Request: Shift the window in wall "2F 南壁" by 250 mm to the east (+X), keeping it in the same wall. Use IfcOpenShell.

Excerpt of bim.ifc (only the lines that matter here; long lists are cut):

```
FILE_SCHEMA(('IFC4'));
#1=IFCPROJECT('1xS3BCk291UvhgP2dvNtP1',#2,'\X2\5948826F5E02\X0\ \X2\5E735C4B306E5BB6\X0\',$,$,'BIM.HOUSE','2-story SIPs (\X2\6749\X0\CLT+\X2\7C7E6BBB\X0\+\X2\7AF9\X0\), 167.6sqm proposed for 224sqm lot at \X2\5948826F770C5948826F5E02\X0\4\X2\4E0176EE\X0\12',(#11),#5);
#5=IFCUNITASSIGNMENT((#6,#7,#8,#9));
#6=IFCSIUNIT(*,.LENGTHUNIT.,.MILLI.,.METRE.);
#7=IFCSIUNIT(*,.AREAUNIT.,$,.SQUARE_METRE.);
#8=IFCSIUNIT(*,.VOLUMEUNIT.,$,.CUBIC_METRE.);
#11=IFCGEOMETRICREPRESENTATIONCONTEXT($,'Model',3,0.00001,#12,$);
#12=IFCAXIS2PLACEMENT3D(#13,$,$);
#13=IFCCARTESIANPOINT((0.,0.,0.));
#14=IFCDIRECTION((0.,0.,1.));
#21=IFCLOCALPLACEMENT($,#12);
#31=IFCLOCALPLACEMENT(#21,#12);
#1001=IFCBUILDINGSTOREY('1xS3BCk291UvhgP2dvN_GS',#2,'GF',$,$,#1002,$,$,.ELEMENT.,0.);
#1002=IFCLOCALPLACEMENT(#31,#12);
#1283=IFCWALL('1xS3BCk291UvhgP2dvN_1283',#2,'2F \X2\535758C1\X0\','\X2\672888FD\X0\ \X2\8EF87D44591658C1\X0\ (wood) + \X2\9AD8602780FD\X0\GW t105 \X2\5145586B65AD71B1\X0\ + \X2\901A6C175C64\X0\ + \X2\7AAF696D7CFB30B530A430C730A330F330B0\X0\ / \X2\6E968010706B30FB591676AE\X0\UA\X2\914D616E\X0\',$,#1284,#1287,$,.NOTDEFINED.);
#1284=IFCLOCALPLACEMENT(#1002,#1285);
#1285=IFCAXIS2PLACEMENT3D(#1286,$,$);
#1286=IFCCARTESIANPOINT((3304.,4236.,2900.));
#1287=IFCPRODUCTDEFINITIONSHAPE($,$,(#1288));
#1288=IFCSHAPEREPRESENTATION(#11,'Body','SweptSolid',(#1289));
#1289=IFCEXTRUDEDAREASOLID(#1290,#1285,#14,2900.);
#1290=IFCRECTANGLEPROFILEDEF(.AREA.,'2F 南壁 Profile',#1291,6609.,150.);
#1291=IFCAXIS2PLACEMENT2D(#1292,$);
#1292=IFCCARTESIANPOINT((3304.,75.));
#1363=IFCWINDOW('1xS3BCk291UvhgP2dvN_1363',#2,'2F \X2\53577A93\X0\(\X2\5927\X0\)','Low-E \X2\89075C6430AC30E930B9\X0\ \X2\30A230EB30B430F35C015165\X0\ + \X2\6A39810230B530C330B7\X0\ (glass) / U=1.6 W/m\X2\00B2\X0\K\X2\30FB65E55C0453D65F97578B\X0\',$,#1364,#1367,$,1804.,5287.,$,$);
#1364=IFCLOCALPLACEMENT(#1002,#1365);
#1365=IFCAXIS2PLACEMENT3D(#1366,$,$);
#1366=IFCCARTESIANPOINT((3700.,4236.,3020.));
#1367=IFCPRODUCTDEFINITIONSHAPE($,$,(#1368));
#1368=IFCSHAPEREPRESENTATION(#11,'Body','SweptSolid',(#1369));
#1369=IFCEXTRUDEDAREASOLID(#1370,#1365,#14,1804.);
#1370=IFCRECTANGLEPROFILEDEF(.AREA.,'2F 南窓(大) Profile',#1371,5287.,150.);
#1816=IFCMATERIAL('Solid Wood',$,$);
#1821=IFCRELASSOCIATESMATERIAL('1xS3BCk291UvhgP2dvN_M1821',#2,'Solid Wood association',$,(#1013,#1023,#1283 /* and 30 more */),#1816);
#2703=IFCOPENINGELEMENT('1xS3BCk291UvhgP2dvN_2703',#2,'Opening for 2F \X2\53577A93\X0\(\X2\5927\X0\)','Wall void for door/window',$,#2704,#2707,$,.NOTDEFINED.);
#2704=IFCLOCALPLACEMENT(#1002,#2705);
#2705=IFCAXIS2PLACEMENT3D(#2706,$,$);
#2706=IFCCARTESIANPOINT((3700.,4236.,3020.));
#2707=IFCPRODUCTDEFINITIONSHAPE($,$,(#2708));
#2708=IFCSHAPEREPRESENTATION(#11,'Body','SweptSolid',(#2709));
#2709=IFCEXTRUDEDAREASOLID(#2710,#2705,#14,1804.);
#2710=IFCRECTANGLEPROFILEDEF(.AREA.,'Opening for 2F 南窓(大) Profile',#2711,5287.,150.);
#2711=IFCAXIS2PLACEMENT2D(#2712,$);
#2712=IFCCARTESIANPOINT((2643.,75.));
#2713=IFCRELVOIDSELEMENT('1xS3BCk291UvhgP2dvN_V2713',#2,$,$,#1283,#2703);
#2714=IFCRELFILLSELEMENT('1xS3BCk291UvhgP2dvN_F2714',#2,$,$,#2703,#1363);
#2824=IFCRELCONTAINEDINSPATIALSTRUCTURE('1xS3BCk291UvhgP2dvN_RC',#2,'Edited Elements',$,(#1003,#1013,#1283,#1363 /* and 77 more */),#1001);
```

```python
import ifcopenshell
import ifcopenshell.api.geometry
import ifcopenshell.util.placement

model = ifcopenshell.open("bim.ifc")

window = model.by_id(1363)
opening = window.FillsVoids[0].RelatingOpeningElement
wall = opening.VoidsElements[0].RelatingBuildingElement

wall_matrix = ifcopenshell.util.placement.get_local_placement(wall.ObjectPlacement)
shift = wall_matrix[:3, 0] * 250.0
before = ifcopenshell.util.placement.get_local_placement(window.ObjectPlacement)[:3, 3].copy()

# The window is not placed relative to its opening, so move both.
for product in (opening, window):
    matrix = ifcopenshell.util.placement.get_local_placement(product.ObjectPlacement)
    matrix[:3, 3] += shift
    ifcopenshell.api.geometry.edit_object_placement(model, product=product, matrix=matrix, is_si=False)

after = ifcopenshell.util.placement.get_local_placement(window.ObjectPlacement)[:3, 3]
print("window moved by", (after - before).round(3) + 0.0)

model.write("bim_rev.ifc")
```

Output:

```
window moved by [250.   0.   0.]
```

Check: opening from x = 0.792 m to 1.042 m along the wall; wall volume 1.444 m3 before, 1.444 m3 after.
